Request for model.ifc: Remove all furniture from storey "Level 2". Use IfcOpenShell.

First a look at what the model holds.

```python
import ifcopenshell
import ifcopenshell.util.element

model = ifcopenshell.open("model.ifc")
print(model.schema)
storey = next(s for s in model.by_type("IfcBuildingStorey") if s.Name == "Level 2")
furniture = [e for e in ifcopenshell.util.element.get_decomposition(storey) if e.is_a("IfcFurnishingElement")]
seen = {}
for e in furniture:
    element_type = ifcopenshell.util.element.get_type(e)
    name = element_type.Name if element_type not in (None, e) else None
    seen[name] = seen.get(name, 0) + 1
for name, count in sorted(seen.items(), key=str):
    print(count, "x", name)
```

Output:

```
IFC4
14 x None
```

```python
import ifcopenshell
import ifcopenshell.api.root
import ifcopenshell.util.element

model = ifcopenshell.open("model.ifc")

storey = next(s for s in model.by_type("IfcBuildingStorey") if s.Name == "Level 2")
furniture = [e for e in ifcopenshell.util.element.get_decomposition(storey) if e.is_a("IfcFurnishingElement")]

for e in furniture:
    ifcopenshell.api.root.remove_product(model, product=e)
print(len(furniture), "removed")

model.write("model_updated.ifc")
```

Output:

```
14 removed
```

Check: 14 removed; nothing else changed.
